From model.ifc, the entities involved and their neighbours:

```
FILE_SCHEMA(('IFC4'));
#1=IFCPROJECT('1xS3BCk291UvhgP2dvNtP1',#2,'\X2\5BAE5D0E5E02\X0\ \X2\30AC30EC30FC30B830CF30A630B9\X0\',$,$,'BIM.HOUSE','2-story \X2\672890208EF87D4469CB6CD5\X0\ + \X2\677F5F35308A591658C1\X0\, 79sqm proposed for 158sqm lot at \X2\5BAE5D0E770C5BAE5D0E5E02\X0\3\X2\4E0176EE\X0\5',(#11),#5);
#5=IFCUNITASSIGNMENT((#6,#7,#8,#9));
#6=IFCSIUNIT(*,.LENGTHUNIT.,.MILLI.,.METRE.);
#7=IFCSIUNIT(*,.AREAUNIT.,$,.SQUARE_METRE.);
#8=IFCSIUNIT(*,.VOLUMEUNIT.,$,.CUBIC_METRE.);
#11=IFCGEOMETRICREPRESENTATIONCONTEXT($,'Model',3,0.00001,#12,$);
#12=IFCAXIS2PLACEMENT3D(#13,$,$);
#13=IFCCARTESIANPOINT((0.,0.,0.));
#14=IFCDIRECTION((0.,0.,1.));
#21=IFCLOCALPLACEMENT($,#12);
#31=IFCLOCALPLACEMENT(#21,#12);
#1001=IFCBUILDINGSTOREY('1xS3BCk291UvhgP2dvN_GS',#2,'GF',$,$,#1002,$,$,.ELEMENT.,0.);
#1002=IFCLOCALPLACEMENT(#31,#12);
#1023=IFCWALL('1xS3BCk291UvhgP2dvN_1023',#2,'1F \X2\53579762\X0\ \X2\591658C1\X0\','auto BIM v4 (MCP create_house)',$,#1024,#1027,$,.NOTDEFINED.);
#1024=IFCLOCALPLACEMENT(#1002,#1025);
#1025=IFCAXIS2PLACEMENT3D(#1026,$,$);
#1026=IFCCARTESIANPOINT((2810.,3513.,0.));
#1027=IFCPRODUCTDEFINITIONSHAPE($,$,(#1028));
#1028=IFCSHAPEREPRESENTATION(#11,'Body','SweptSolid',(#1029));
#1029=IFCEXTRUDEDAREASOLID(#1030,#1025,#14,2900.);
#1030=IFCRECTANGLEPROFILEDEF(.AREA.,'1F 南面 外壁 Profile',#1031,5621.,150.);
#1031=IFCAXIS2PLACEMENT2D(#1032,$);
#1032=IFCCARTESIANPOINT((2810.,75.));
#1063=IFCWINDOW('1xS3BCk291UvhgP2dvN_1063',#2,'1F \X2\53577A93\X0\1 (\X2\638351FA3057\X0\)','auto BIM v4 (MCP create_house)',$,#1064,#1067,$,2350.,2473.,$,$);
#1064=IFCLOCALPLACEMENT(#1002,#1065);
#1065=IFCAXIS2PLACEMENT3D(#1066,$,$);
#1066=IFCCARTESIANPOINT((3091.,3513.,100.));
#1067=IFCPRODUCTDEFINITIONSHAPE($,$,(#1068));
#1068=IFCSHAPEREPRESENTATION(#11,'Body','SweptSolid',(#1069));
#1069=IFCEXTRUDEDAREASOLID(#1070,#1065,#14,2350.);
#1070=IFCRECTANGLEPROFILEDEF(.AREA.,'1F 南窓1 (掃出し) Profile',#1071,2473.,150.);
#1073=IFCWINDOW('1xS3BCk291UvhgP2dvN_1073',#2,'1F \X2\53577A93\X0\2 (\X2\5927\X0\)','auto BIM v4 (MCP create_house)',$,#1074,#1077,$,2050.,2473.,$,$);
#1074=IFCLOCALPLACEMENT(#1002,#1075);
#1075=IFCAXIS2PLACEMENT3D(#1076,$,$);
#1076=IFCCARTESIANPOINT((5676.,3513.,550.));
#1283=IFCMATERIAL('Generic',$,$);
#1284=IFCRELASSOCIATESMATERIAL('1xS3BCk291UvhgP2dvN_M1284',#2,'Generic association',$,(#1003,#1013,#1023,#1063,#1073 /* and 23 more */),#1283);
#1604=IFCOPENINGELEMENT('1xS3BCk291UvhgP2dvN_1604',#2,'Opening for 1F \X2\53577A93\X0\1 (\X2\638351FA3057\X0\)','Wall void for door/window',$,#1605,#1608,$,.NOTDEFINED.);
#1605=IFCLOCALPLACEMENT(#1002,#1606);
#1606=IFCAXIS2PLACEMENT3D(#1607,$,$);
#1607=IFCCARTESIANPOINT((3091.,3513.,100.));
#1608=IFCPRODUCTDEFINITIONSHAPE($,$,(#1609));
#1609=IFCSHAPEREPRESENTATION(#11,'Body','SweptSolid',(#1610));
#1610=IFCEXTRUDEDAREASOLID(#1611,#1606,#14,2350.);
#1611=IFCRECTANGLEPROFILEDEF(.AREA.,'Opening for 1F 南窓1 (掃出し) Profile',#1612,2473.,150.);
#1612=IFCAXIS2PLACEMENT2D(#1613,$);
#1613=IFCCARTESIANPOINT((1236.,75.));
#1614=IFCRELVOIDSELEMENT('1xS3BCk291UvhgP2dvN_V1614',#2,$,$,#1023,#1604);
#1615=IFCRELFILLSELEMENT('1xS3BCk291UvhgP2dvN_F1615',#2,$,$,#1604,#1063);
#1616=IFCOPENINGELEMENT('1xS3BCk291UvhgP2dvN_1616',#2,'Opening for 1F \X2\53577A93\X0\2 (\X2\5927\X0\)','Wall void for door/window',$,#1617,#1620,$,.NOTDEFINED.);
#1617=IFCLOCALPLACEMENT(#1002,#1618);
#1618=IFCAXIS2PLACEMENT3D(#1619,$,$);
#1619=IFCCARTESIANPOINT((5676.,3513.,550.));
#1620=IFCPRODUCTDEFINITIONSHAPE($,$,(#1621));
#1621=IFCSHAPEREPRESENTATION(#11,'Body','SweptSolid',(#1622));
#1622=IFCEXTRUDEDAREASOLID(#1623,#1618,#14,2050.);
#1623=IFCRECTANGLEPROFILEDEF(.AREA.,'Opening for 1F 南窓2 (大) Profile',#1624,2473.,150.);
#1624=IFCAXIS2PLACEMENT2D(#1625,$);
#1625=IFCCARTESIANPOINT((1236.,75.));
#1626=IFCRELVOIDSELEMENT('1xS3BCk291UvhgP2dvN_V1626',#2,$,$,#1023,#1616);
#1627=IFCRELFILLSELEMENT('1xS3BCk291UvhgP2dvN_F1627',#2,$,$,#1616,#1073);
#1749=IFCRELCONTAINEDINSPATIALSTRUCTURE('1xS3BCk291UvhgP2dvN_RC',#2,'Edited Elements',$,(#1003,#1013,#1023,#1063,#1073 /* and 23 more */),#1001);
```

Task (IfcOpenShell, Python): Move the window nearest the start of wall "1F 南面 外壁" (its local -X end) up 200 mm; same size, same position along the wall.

```python
import numpy as np
import ifcopenshell
import ifcopenshell.api.geometry
import ifcopenshell.util.placement
import ifcopenshell.util.unit

model = ifcopenshell.open("model.ifc")
unit_scale = ifcopenshell.util.unit.calculate_unit_scale(model)

window = model.by_id(1063)
opening = window.FillsVoids[0].RelatingOpeningElement
dz = 200.0

shift = np.array([0.0, 0.0, dz])
# The window is not placed relative to its opening, so move both.
for product in (opening, window):
    matrix = ifcopenshell.util.placement.get_local_placement(product.ObjectPlacement)
    matrix[:3, 3] += shift
    ifcopenshell.api.geometry.edit_object_placement(model, product=product, matrix=matrix, is_si=False)

print(f"moved by {dz * unit_scale:+.3f} m")

model.write("model-out.ifc")
```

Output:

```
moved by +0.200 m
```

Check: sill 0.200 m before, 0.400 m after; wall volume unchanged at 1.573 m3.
